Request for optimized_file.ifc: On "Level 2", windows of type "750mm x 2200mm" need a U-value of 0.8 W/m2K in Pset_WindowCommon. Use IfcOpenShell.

First a look at what the model holds.

```python
import ifcopenshell
import ifcopenshell.util.element

model = ifcopenshell.open("optimized_file.ifc")
print(model.schema)
storey = next(s for s in model.by_type("IfcBuildingStorey") if s.Name == "Level 2")
windows = [e for e in ifcopenshell.util.element.get_decomposition(storey) if e.is_a("IfcWindow")]
seen = {}
for e in windows:
    element_type = ifcopenshell.util.element.get_type(e)
    key = (element_type.Name if element_type != e and element_type else None, ifcopenshell.util.element.get_pset(e, "Pset_WindowCommon", "ThermalTransmittance"))
    seen[key] = seen.get(key, 0) + 1
for (name, value), count in sorted(seen.items(), key=str):
    print(count, "x", name, "|", value)
```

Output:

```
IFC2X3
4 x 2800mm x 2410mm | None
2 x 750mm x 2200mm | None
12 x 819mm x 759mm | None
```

```python
import ifcopenshell
import ifcopenshell.api.pset
import ifcopenshell.util.element

model = ifcopenshell.open("optimized_file.ifc")

storey = next(s for s in model.by_type("IfcBuildingStorey") if s.Name == "Level 2")
windows = [e for e in ifcopenshell.util.element.get_decomposition(storey) if e.is_a("IfcWindow")]

count = 0
for e in windows:
    element_type = ifcopenshell.util.element.get_type(e)
    if element_type in (None, e) or element_type.Name != "750mm x 2200mm":
        continue
    # add_pset returns the element's existing set when there is one.
    pset = ifcopenshell.api.pset.add_pset(model, product=e, name="Pset_WindowCommon")
    ifcopenshell.api.pset.edit_pset(model, pset=pset, properties={"ThermalTransmittance": 0.8})
    count += 1

print(count, "windows updated")

model.write("optimized_file-out.ifc")
```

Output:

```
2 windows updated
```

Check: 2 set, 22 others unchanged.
